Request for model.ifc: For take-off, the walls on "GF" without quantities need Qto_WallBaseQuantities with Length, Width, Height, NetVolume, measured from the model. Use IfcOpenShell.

First a look at what the model holds.

```python
import ifcopenshell
import ifcopenshell.util.element
import ifcopenshell.util.unit

model = ifcopenshell.open("model.ifc")
print(model.schema)
for unit_type in ("LENGTHUNIT", "AREAUNIT", "VOLUMEUNIT"):
    print(unit_type, ifcopenshell.util.unit.calculate_unit_scale(model, unit_type))
storey = next(s for s in model.by_type("IfcBuildingStorey") if s.Name == "GF")
walls = [e for e in ifcopenshell.util.element.get_decomposition(storey) if e.is_a("IfcWall")]
for e in sorted(walls, key=lambda e: e.id()):
    print(e.id(), e.is_a(), e.Name, list(ifcopenshell.util.element.get_psets(e, qtos_only=True)), sep=" | ")
```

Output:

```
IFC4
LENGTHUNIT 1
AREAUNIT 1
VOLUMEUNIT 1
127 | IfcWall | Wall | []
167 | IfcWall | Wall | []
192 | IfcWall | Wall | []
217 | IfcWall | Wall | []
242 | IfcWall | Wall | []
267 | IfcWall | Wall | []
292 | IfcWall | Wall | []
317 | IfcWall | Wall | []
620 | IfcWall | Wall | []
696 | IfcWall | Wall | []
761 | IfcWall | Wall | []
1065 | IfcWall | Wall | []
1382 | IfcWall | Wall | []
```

```python
import ifcopenshell
import ifcopenshell.api.pset
import ifcopenshell.geom
import ifcopenshell.util.element
import ifcopenshell.util.shape
import ifcopenshell.util.unit

model = ifcopenshell.open("model.ifc")
unit_scale = ifcopenshell.util.unit.calculate_unit_scale(model)
volume_scale = ifcopenshell.util.unit.calculate_unit_scale(model, "VOLUMEUNIT")
settings = ifcopenshell.geom.settings()

storey = next(s for s in model.by_type("IfcBuildingStorey") if s.Name == "GF")
walls = [e for e in ifcopenshell.util.element.get_decomposition(storey) if e.is_a("IfcWall")]

for e in sorted(walls, key=lambda e: e.id()):
    if ifcopenshell.util.element.get_psets(e, qtos_only=True, should_inherit=False):
        continue
    # Geometry comes back in metres, in the element's own axes.
    shape = ifcopenshell.geom.create_shape(settings, e)
    values = {
        "Length": ifcopenshell.util.shape.get_x(shape.geometry) / unit_scale,
        "Width": ifcopenshell.util.shape.get_y(shape.geometry) / unit_scale,
        "Height": ifcopenshell.util.shape.get_z(shape.geometry) / unit_scale,
        "NetVolume": ifcopenshell.util.shape.get_volume(shape.geometry) / volume_scale,
    }
    qto = ifcopenshell.api.pset.add_qto(model, product=e, name="Qto_WallBaseQuantities")
    ifcopenshell.api.pset.edit_qto(model, qto=qto, properties=values)
    print(e.id(), {k: round(v, 3) for k, v in values.items()})

model.write("model_edited.ifc")
```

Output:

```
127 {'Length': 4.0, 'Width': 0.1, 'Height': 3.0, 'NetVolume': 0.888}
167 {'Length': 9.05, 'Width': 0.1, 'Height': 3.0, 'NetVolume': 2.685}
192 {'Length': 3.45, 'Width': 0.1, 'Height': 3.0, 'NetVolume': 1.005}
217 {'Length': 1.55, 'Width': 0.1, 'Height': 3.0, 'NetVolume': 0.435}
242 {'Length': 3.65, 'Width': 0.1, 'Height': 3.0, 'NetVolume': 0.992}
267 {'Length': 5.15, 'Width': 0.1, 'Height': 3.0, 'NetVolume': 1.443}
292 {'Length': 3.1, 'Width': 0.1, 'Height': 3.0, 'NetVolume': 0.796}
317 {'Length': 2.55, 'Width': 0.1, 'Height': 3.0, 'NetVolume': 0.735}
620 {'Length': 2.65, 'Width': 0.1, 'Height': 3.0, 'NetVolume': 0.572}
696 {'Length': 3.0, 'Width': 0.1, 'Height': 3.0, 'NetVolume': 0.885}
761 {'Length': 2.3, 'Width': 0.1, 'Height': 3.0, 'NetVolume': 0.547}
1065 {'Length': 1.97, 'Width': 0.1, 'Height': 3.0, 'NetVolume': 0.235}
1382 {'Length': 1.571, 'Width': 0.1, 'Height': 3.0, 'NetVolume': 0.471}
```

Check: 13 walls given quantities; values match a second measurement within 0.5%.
